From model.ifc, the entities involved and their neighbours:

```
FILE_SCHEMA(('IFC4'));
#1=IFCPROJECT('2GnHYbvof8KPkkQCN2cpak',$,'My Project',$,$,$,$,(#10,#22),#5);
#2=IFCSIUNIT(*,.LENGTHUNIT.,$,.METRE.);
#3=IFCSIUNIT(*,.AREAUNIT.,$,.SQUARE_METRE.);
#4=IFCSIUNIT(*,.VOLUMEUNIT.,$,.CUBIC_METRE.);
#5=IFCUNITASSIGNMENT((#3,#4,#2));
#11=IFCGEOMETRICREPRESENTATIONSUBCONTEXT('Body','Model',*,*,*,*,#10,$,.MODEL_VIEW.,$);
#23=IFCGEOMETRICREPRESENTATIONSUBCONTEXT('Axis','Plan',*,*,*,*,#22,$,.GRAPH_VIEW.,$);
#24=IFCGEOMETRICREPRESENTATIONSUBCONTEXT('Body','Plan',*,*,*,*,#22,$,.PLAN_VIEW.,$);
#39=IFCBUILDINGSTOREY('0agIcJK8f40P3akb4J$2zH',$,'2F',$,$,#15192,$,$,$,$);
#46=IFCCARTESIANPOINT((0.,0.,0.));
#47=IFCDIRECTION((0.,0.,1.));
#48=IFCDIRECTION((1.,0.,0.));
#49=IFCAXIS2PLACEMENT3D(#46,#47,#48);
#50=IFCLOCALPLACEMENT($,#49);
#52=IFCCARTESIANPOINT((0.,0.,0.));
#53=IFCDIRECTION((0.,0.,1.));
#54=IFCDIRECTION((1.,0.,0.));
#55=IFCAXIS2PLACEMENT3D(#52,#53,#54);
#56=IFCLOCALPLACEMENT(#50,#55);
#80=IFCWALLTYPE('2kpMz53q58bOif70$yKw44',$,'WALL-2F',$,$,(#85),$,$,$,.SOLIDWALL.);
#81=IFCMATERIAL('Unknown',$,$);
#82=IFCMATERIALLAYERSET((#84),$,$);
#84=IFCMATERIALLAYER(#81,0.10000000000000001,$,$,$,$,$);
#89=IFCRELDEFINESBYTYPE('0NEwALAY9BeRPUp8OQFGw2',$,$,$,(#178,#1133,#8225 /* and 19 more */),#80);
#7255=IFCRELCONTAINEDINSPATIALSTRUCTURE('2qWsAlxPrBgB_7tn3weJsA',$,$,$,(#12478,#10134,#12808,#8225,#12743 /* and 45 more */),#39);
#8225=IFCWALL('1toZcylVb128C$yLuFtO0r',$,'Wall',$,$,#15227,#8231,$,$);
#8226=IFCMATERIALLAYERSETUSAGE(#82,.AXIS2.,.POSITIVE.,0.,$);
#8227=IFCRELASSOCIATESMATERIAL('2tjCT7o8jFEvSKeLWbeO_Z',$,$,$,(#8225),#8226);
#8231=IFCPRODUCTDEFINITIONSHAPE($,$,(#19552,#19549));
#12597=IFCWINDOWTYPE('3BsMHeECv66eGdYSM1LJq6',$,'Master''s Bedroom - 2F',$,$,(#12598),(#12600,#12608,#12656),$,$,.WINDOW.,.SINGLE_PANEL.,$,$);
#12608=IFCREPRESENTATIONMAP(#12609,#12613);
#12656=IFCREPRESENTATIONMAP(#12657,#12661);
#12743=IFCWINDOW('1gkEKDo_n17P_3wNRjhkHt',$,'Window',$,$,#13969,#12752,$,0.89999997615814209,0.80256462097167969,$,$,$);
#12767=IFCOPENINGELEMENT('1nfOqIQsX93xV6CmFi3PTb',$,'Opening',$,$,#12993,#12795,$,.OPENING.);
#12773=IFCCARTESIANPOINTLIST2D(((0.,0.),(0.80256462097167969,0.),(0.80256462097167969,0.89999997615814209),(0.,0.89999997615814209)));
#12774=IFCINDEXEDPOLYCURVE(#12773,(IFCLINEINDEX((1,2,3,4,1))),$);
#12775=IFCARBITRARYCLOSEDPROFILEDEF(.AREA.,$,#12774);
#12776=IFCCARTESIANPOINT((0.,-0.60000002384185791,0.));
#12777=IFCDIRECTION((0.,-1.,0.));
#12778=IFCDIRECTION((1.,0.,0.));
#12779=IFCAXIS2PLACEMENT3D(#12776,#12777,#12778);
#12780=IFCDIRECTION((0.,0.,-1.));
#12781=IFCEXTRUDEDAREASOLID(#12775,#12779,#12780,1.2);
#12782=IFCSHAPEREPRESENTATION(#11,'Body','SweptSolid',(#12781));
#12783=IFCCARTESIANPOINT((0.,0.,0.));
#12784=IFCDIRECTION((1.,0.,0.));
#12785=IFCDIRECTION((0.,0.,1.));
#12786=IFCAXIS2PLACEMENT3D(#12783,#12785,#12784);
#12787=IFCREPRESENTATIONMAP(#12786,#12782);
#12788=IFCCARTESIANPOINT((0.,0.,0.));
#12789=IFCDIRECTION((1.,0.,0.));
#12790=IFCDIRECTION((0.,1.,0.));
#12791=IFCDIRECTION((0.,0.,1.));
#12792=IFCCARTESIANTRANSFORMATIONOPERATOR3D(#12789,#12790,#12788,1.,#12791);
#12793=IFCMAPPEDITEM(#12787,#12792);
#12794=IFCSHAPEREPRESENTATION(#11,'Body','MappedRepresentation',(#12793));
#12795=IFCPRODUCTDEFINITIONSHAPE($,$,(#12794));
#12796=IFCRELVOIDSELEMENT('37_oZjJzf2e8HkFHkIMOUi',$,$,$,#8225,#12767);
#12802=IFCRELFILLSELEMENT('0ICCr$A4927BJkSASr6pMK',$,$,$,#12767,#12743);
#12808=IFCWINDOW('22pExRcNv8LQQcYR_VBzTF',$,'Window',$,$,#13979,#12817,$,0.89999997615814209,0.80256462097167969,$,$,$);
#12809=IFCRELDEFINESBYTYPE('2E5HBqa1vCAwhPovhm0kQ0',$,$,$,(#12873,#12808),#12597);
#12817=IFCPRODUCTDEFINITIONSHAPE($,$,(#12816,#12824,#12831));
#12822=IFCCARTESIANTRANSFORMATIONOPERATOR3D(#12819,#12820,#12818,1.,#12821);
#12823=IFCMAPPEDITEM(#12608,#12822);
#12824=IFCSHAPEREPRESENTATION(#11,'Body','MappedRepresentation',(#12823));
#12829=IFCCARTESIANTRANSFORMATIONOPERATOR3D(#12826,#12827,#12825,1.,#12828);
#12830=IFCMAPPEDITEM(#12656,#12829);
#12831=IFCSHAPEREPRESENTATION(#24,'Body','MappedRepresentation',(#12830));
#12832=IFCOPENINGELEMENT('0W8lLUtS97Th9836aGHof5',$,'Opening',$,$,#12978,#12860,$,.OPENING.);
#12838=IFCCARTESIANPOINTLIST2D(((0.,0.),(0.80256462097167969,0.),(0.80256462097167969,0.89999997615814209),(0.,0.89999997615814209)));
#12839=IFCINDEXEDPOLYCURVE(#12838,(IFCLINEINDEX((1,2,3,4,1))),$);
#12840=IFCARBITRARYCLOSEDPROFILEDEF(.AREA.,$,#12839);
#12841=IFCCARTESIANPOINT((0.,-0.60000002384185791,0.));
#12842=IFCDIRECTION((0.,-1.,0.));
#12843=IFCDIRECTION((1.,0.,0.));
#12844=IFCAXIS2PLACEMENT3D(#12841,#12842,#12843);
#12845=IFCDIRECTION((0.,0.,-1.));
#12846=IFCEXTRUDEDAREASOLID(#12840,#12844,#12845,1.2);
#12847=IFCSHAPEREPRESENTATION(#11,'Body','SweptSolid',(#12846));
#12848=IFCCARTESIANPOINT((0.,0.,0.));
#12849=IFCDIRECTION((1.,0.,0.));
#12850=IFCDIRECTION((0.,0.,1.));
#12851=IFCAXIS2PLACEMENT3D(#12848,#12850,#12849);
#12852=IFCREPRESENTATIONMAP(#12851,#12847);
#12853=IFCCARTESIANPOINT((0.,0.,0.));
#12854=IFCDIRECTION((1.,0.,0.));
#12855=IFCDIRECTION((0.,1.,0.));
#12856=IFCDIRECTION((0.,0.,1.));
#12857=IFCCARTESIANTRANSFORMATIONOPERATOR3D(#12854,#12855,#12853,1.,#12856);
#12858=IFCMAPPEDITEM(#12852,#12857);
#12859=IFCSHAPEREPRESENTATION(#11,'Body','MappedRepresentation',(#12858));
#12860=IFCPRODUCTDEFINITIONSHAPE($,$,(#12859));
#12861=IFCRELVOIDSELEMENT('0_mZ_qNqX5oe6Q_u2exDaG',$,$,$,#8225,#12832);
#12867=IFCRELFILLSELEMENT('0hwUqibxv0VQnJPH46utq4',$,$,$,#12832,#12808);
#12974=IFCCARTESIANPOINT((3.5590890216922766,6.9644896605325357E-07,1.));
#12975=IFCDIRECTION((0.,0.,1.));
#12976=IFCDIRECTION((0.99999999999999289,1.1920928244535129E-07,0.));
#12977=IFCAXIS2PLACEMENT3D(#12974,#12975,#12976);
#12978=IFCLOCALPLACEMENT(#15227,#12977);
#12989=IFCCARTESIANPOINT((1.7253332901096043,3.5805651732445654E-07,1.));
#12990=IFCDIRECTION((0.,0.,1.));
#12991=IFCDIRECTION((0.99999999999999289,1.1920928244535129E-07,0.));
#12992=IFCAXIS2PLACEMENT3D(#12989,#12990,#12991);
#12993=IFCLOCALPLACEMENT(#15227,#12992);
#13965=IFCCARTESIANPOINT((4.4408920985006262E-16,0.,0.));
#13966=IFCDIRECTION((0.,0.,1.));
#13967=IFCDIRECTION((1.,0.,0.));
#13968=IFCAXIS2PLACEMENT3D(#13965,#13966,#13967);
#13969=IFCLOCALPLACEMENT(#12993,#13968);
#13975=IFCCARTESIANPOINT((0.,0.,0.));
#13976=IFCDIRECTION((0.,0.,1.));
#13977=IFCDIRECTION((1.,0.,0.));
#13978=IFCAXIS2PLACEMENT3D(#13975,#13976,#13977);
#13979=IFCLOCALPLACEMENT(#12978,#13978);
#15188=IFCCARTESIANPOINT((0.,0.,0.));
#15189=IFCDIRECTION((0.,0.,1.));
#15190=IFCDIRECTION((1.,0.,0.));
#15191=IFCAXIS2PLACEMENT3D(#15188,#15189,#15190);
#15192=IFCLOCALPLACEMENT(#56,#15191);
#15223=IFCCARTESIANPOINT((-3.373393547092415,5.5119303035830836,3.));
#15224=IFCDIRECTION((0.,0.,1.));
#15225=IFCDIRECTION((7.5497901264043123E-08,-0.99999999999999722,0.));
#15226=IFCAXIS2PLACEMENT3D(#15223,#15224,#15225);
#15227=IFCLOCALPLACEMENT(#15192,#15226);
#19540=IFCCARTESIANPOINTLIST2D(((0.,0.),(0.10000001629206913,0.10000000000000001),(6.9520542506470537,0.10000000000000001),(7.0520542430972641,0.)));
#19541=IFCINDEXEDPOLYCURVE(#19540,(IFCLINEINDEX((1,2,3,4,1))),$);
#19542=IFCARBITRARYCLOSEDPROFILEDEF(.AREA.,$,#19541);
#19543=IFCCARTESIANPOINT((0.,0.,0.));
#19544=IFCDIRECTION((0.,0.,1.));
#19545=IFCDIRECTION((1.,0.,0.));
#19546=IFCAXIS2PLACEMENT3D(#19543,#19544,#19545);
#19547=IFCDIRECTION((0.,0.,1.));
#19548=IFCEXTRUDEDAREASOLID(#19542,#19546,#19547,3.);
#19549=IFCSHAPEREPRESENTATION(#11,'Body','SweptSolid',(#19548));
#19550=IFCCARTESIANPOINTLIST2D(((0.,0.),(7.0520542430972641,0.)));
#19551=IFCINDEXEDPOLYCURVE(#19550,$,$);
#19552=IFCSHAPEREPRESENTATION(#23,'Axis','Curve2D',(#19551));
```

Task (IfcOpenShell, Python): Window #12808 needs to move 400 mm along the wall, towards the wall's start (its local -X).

```python
import ifcopenshell
import ifcopenshell.api.geometry
import ifcopenshell.util.placement
import ifcopenshell.util.unit

model = ifcopenshell.open("model.ifc")
unit_scale = ifcopenshell.util.unit.calculate_unit_scale(model)

window = model.by_guid("22pExRcNv8LQQcYR_VBzTF")
opening = window.FillsVoids[0].RelatingOpeningElement
wall = opening.VoidsElements[0].RelatingBuildingElement

wall_matrix = ifcopenshell.util.placement.get_local_placement(wall.ObjectPlacement)
shift = wall_matrix[:3, 0] * -0.4 / unit_scale
before = ifcopenshell.util.placement.get_local_placement(window.ObjectPlacement)[:3, 3].copy()

# The window is placed relative to its opening, so it follows when the opening moves.
matrix = ifcopenshell.util.placement.get_local_placement(opening.ObjectPlacement)
matrix[:3, 3] += shift
ifcopenshell.api.geometry.edit_object_placement(
    model, product=opening, matrix=matrix, is_si=False, should_transform_children=True
)

after = ifcopenshell.util.placement.get_local_placement(window.ObjectPlacement)[:3, 3]
print("window moved by", (after - before).round(3) + 0.0)

model.write("model_updated.ifc")
```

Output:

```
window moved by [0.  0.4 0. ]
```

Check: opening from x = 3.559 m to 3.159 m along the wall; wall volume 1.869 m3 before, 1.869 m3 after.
